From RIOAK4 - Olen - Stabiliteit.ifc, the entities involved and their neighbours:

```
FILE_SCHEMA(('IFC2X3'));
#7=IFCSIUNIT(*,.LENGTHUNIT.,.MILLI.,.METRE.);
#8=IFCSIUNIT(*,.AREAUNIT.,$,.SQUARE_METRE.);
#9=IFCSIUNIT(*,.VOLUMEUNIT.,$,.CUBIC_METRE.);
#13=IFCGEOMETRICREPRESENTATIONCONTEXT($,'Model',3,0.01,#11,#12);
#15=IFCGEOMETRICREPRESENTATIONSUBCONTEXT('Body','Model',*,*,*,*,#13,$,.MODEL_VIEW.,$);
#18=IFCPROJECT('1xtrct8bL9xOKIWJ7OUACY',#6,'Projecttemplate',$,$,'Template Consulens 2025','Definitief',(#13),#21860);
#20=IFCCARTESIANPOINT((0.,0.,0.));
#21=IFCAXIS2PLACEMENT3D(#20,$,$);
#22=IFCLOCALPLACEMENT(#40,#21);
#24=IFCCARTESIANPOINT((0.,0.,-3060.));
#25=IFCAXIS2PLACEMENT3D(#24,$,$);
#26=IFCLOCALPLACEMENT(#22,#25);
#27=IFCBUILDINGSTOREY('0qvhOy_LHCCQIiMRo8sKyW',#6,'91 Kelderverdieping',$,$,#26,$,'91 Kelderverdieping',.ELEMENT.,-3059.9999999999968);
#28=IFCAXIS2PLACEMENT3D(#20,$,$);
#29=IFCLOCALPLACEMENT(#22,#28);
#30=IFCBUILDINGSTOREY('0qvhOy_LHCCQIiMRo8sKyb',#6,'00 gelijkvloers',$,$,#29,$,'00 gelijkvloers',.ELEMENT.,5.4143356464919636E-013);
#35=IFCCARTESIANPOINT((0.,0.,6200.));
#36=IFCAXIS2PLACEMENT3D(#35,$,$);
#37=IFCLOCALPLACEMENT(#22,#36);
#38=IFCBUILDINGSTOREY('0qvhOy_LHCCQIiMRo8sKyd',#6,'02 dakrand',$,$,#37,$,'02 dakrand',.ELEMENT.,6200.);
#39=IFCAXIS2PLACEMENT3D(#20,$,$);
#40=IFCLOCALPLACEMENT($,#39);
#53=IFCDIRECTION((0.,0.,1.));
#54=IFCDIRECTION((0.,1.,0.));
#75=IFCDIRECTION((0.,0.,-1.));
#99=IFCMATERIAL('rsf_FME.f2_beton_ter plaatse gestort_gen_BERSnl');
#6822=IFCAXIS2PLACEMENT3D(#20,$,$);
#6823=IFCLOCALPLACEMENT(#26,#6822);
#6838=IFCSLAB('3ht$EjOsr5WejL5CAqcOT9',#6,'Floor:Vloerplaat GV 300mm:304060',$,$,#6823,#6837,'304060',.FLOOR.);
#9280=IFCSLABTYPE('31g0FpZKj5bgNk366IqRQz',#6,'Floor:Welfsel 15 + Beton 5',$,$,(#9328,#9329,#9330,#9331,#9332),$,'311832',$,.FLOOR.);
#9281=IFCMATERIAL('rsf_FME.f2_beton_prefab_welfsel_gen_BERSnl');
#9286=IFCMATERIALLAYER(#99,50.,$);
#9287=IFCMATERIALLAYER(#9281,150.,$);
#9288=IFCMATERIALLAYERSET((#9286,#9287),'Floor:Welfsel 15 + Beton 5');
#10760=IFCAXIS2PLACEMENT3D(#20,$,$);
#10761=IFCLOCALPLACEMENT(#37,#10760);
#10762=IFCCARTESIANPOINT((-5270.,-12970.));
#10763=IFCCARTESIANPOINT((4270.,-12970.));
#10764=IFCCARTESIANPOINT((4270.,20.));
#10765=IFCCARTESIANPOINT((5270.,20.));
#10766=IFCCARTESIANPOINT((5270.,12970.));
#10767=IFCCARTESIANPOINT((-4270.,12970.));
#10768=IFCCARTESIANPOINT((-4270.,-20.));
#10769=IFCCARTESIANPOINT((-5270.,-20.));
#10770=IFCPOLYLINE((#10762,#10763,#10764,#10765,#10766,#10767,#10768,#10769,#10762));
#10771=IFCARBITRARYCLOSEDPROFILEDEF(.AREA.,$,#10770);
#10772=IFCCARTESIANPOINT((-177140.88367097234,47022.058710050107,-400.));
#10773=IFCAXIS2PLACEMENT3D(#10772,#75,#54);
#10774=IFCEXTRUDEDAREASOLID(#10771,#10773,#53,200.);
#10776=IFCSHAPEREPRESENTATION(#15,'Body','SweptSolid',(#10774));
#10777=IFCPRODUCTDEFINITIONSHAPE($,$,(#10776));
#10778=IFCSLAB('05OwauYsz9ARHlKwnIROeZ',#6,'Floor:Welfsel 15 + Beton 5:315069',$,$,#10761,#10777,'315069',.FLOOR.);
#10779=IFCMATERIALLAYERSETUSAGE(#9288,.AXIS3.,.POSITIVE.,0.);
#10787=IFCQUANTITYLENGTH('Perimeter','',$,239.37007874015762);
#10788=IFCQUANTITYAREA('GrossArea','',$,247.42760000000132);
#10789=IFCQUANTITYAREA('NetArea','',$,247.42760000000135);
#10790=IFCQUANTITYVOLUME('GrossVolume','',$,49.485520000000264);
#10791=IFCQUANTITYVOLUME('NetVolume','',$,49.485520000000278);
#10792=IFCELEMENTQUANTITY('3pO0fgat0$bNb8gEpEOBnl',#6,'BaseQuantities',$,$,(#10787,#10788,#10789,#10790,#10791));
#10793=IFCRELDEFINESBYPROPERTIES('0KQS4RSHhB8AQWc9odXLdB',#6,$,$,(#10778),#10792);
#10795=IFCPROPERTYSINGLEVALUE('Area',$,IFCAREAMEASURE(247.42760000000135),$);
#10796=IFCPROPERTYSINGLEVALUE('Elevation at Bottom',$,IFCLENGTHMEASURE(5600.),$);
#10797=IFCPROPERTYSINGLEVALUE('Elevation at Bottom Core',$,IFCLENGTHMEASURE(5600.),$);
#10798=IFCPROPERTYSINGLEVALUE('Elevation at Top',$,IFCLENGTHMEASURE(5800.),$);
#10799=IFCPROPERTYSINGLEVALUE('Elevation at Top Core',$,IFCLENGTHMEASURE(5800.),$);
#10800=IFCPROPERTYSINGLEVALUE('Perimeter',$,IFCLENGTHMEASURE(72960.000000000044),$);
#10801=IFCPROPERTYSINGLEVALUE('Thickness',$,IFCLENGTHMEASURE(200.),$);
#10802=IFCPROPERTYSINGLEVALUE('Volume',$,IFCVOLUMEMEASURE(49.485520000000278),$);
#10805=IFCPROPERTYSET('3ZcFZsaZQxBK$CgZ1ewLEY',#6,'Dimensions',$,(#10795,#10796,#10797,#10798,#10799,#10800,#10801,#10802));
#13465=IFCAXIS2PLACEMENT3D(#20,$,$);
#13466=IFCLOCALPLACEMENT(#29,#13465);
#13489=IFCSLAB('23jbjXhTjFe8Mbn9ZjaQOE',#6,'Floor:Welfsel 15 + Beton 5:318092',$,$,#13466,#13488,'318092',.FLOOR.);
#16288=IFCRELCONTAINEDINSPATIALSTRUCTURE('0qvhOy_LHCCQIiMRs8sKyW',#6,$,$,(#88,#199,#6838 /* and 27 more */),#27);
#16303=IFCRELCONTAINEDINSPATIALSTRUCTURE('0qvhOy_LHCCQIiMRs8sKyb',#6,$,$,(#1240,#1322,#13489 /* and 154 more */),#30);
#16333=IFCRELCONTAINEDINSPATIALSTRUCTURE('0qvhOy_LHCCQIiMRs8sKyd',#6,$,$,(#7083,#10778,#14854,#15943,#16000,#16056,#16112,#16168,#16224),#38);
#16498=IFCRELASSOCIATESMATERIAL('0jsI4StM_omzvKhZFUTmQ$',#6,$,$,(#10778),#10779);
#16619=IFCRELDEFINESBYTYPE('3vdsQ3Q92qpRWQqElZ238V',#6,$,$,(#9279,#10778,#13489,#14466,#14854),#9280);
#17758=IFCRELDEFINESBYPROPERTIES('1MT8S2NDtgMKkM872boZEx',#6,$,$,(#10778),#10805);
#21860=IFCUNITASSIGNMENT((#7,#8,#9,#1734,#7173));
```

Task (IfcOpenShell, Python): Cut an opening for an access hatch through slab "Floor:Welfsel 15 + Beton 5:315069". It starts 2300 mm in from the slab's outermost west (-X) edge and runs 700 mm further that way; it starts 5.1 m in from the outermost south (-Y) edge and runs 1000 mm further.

```python
import numpy as np
import ifcopenshell
import ifcopenshell.api.feature
import ifcopenshell.api.geometry
import ifcopenshell.api.pset
import ifcopenshell.api.root
import ifcopenshell.geom
import ifcopenshell.util.element
import ifcopenshell.util.placement
import ifcopenshell.util.representation
import ifcopenshell.util.shape
import ifcopenshell.util.unit

model = ifcopenshell.open("RIOAK4 - Olen - Stabiliteit.ifc")
unit_scale = ifcopenshell.util.unit.calculate_unit_scale(model)
area_scale = ifcopenshell.util.unit.calculate_unit_scale(model, "AREAUNIT")
volume_scale = ifcopenshell.util.unit.calculate_unit_scale(model, "VOLUMEUNIT")
settings = ifcopenshell.geom.settings()


def volume(element):
    """Net volume in cubic metres, openings subtracted."""
    shape = ifcopenshell.geom.create_shape(settings, element)
    return ifcopenshell.util.shape.get_volume(shape.geometry)


slab = model.by_guid("05OwauYsz9ARHlKwnIROeZ")
before = volume(slab)

# Extent in the slab's own axes, in metres. The edges named are its -X and -Y sides.
slab_shape = ifcopenshell.geom.create_shape(settings, slab)
vertices = ifcopenshell.util.shape.get_vertices(slab_shape.geometry)
x_min, y_min, bottom = vertices.min(axis=0)
top = vertices[:, 2].max()

opening = ifcopenshell.api.root.create_entity(model, ifc_class="IfcOpeningElement", name="Access hatch opening")
context = ifcopenshell.util.representation.get_context(model, "Model", "Body", "MODEL_VIEW")
width, depth = 0.7, 1
outline = [(0.0, 0.0), (width, 0.0), (width, depth), (0.0, depth), (0.0, 0.0)]
# Overshoot both faces by 50 mm so the cut is clean.
shape = ifcopenshell.api.geometry.add_slab_representation(
    model, context=context, depth=top - bottom + 0.1, polyline=outline
)
ifcopenshell.api.geometry.assign_representation(model, product=opening, representation=shape)

matrix = ifcopenshell.util.placement.get_local_placement(slab.ObjectPlacement)
matrix[:, 3] = matrix @ np.append(np.array([x_min + 2.3, y_min + 5.1, bottom - 0.05]) / unit_scale, 1.0)
ifcopenshell.api.geometry.edit_object_placement(model, product=opening, matrix=matrix, is_si=False)
ifcopenshell.api.feature.add_feature(model, feature=opening, element=slab)

after = volume(slab)

# Update the slab's stored quantities.
qto = model.by_id(ifcopenshell.util.element.get_pset(slab, "BaseQuantities", should_inherit=False)["id"])
ifcopenshell.api.pset.edit_qto(model, qto=qto, properties={
    "NetArea": after / (top - bottom) / area_scale,
    "NetVolume": after / volume_scale,
})
pset = model.by_id(ifcopenshell.util.element.get_pset(slab, "Dimensions", should_inherit=False)["id"])
ifcopenshell.api.pset.edit_pset(model, pset=pset, properties={
    "Area": model.create_entity("IfcAreaMeasure", after / (top - bottom) / area_scale),
    "Volume": model.create_entity("IfcVolumeMeasure", after / volume_scale),
})

print(f"slab volume {before:.3f} -> {after:.3f} m3")

model.write("RIOAK4 - Olen - Stabiliteit_edited.ifc")
```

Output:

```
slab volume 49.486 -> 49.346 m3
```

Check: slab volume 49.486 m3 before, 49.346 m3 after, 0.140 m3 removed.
